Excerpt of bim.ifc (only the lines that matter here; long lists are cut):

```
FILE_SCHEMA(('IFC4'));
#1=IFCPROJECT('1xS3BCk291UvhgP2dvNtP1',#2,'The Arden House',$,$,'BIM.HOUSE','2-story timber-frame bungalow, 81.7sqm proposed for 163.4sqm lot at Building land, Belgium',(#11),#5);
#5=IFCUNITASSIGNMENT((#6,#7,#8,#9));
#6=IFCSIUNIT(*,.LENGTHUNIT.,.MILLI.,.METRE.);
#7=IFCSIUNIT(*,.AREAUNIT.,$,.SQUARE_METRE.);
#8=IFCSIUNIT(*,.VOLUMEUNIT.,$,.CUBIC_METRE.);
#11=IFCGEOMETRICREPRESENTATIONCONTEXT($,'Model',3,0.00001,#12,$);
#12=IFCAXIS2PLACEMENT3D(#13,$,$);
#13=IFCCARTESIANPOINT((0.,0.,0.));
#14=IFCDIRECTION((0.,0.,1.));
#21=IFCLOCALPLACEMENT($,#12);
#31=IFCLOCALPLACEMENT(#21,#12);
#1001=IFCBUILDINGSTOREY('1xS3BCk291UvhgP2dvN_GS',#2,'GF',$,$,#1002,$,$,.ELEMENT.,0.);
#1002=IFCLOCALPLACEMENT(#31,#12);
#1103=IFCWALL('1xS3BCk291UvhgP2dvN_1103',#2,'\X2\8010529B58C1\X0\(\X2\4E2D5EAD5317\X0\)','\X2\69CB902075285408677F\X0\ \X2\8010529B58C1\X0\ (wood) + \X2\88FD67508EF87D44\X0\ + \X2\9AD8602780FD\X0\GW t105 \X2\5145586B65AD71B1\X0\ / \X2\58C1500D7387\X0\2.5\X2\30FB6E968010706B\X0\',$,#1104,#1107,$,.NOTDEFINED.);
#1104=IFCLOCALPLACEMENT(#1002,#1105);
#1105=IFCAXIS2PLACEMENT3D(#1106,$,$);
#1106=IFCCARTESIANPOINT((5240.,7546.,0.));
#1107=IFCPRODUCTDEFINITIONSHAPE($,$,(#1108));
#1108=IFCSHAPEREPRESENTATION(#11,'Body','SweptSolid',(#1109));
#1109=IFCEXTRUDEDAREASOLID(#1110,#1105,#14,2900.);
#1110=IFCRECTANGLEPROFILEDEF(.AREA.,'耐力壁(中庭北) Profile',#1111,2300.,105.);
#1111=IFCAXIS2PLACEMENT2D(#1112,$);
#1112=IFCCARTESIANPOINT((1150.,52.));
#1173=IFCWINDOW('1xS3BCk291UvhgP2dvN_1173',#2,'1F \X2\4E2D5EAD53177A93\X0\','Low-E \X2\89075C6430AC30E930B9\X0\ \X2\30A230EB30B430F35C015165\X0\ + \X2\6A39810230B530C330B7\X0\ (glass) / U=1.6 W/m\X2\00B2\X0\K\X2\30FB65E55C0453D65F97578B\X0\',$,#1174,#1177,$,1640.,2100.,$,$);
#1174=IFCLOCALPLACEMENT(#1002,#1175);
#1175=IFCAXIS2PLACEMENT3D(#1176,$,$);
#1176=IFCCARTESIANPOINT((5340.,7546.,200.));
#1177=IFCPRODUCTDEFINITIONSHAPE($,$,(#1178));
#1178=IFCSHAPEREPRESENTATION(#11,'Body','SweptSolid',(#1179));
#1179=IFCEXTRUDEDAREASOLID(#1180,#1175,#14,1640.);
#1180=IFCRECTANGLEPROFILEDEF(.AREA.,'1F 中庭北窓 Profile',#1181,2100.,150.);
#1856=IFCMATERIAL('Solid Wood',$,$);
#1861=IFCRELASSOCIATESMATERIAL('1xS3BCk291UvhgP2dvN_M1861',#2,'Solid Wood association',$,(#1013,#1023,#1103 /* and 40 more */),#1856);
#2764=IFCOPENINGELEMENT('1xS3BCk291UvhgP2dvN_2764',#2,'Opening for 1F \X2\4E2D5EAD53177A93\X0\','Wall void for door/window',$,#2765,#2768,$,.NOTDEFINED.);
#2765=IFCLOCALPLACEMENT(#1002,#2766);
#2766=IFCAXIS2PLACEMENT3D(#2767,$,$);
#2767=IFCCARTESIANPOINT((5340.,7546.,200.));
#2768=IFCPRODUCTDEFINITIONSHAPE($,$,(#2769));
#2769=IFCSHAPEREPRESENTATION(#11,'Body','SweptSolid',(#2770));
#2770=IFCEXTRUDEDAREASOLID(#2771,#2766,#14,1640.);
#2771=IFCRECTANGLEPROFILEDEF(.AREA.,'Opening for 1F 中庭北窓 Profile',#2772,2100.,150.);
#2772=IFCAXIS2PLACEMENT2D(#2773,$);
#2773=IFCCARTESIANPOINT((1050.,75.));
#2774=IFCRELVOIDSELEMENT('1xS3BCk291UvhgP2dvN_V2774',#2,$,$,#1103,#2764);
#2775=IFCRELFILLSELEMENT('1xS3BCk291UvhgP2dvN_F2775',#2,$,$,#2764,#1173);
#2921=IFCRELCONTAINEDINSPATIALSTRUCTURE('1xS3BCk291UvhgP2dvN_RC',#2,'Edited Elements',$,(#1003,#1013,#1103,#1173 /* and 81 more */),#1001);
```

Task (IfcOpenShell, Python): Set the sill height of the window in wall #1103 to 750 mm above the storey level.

```python
import numpy as np
import ifcopenshell
import ifcopenshell.api.geometry
import ifcopenshell.geom
import ifcopenshell.util.element
import ifcopenshell.util.placement
import ifcopenshell.util.shape
import ifcopenshell.util.unit

model = ifcopenshell.open("bim.ifc")
unit_scale = ifcopenshell.util.unit.calculate_unit_scale(model)

window = model.by_id(1173)
opening = window.FillsVoids[0].RelatingOpeningElement
storey = ifcopenshell.util.element.get_container(window, ifc_class="IfcBuildingStorey")
level = ifcopenshell.util.placement.get_local_placement(storey.ObjectPlacement)[2, 3]

# The opening's origin need not be at the sill, so measure its lowest point.
shape = ifcopenshell.geom.create_shape(ifcopenshell.geom.settings(), opening)
bottom = ifcopenshell.util.shape.get_shape_bottom_elevation(shape, shape.geometry) / unit_scale
dz = level + 750.0 - bottom

shift = np.array([0.0, 0.0, dz])
# The window is not placed relative to its opening, so move both.
for product in (opening, window):
    matrix = ifcopenshell.util.placement.get_local_placement(product.ObjectPlacement)
    matrix[:3, 3] += shift
    ifcopenshell.api.geometry.edit_object_placement(model, product=product, matrix=matrix, is_si=False)

print(f"moved by {dz * unit_scale:+.3f} m")

model.write("bim_v2.ifc")
```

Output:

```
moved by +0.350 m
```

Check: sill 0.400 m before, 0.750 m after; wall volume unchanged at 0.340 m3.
